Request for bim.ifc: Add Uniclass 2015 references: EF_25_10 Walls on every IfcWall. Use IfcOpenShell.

First a look at what the model holds.

```python
import ifcopenshell

model = ifcopenshell.open("bim.ifc")
print(model.schema)
print("classifications:", [c.Name for c in model.by_type("IfcClassification")])
for ifc_class in ("IfcDoor", "IfcRoof", "IfcStair", "IfcWall", "IfcWindow"):
    print(ifc_class, len(model.by_type(ifc_class)))
```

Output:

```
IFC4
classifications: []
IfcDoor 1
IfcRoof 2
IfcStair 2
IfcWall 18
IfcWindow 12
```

```python
import ifcopenshell
import ifcopenshell.api.classification

model = ifcopenshell.open("bim.ifc")

system = ifcopenshell.api.classification.add_classification(model, classification="Uniclass 2015")

codes = {
    "IfcWall": ("EF_25_10", "Walls"),
}
for ifc_class, (code, name) in codes.items():
    products = model.by_type(ifc_class)
    ifcopenshell.api.classification.add_reference(
        model, products=products, classification=system, identification=code, name=name
    )
    print(code, len(products))

model.write("bim-out.ifc")
```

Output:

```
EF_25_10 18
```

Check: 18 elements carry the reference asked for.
